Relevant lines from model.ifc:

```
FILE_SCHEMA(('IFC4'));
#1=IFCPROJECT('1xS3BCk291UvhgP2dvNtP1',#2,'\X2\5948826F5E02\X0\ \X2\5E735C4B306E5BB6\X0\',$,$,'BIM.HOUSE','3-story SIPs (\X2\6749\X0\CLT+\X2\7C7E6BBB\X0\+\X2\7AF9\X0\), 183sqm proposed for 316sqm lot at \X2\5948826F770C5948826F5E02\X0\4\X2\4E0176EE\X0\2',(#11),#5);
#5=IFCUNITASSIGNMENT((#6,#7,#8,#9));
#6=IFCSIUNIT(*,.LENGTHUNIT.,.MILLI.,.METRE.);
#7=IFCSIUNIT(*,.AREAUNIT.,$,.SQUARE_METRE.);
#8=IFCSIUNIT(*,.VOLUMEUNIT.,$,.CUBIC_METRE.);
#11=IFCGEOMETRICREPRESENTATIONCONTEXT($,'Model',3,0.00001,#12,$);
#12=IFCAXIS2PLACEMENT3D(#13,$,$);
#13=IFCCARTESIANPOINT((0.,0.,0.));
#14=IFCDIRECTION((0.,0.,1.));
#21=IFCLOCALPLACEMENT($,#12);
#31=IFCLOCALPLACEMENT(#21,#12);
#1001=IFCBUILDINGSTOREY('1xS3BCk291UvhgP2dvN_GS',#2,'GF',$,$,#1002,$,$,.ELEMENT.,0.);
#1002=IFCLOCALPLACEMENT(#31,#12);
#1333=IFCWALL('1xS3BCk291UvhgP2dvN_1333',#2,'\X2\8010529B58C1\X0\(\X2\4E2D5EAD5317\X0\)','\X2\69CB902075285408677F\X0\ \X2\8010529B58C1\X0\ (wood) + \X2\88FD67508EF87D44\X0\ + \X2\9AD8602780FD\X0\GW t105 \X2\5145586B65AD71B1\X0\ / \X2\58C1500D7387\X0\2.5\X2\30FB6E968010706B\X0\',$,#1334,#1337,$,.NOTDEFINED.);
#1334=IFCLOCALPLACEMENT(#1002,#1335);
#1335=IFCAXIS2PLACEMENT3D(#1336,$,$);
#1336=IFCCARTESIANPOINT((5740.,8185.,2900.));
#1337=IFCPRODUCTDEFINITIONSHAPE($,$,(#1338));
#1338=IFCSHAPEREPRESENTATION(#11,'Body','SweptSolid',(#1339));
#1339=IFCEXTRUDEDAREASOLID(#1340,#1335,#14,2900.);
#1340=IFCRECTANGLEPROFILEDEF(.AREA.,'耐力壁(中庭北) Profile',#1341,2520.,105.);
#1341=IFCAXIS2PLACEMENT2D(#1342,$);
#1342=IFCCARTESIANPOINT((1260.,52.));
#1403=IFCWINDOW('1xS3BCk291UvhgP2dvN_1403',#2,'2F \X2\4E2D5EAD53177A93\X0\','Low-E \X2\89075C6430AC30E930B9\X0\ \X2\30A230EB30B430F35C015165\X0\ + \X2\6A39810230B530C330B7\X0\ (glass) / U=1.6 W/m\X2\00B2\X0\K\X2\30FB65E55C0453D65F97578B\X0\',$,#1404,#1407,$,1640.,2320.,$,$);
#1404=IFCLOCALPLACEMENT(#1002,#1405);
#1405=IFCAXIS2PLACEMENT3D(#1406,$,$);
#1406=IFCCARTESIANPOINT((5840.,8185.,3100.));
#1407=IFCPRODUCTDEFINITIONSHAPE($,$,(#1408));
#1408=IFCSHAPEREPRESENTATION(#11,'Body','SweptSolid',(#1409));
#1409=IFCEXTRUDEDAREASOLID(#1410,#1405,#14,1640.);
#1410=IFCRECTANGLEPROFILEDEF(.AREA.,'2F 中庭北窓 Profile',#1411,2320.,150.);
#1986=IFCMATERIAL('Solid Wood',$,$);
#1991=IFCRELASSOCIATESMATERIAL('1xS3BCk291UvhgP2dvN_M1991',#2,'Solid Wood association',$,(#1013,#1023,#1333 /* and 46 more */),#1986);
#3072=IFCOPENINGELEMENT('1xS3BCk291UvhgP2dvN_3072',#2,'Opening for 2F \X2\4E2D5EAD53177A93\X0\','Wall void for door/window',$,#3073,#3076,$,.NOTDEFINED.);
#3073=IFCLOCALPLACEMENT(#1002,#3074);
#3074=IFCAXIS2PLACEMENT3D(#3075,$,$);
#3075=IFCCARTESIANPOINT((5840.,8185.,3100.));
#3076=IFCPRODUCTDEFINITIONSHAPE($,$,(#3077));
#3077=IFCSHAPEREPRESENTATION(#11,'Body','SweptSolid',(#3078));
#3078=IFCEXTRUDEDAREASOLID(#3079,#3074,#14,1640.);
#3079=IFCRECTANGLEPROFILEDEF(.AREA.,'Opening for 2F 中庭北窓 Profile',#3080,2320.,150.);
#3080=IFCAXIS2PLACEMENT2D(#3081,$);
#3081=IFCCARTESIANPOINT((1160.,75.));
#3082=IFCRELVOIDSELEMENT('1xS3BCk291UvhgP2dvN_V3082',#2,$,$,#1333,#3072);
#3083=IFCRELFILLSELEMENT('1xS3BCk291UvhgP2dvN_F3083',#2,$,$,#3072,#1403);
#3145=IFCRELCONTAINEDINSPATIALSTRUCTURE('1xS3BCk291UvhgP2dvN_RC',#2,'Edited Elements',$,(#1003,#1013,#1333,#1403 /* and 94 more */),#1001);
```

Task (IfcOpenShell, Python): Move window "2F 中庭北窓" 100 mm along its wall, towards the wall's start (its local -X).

```python
import ifcopenshell
import ifcopenshell.api.geometry
import ifcopenshell.util.placement

model = ifcopenshell.open("model.ifc")

window = model.by_id(1403)
opening = window.FillsVoids[0].RelatingOpeningElement
wall = opening.VoidsElements[0].RelatingBuildingElement

wall_matrix = ifcopenshell.util.placement.get_local_placement(wall.ObjectPlacement)
shift = wall_matrix[:3, 0] * -100.0
before = ifcopenshell.util.placement.get_local_placement(window.ObjectPlacement)[:3, 3].copy()

# The window is not placed relative to its opening, so move both.
for product in (opening, window):
    matrix = ifcopenshell.util.placement.get_local_placement(product.ObjectPlacement)
    matrix[:3, 3] += shift
    ifcopenshell.api.geometry.edit_object_placement(model, product=product, matrix=matrix, is_si=False)

after = ifcopenshell.util.placement.get_local_placement(window.ObjectPlacement)[:3, 3]
print("window moved by", (after - before).round(3) + 0.0)

model.write("model_updated.ifc")
```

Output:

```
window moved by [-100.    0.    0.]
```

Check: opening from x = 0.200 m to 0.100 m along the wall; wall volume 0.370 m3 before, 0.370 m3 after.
